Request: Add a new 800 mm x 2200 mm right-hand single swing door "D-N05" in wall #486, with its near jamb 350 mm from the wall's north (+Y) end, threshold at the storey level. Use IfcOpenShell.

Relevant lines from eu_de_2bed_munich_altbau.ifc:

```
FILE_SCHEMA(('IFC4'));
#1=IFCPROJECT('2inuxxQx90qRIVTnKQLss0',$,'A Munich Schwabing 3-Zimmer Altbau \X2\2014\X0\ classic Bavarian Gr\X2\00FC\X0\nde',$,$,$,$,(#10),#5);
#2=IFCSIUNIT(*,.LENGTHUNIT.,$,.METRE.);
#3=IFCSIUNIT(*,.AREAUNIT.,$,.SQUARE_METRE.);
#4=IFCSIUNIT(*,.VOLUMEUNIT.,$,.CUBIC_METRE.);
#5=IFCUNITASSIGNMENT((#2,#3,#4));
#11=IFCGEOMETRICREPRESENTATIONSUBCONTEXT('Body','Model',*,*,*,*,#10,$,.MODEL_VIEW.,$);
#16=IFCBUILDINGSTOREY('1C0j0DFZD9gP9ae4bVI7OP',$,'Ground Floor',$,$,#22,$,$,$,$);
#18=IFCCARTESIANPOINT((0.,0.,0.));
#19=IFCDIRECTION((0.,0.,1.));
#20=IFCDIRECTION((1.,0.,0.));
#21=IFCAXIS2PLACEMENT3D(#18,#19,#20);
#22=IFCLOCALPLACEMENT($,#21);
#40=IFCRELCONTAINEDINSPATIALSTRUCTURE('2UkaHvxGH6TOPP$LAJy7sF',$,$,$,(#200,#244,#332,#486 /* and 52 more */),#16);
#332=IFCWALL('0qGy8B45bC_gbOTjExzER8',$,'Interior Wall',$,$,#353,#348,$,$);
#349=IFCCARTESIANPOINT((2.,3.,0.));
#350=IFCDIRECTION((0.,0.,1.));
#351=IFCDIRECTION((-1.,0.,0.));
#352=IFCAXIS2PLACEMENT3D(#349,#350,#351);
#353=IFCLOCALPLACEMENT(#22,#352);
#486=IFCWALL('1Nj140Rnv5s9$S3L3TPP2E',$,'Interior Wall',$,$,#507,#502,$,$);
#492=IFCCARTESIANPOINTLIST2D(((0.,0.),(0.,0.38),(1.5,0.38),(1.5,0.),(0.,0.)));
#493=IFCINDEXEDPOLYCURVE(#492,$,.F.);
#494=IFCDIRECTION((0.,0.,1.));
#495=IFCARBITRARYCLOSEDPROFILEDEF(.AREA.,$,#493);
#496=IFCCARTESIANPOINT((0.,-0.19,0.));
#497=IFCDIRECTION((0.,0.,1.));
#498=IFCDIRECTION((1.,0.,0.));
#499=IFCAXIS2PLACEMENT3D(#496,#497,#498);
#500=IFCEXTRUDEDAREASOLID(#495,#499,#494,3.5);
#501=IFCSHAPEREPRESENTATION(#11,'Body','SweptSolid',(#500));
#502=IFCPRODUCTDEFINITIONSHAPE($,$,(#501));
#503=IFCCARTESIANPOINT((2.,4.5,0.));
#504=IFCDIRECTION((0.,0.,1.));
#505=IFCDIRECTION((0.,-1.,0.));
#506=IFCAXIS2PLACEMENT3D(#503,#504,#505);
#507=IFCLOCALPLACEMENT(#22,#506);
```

```python
import numpy as np
import ifcopenshell
import ifcopenshell.api.feature
import ifcopenshell.api.geometry
import ifcopenshell.api.root
import ifcopenshell.api.spatial
import ifcopenshell.geom
import ifcopenshell.util.element
import ifcopenshell.util.placement
import ifcopenshell.util.representation
import ifcopenshell.util.shape
import ifcopenshell.util.unit

model = ifcopenshell.open("eu_de_2bed_munich_altbau.ifc")
unit_scale = ifcopenshell.util.unit.calculate_unit_scale(model)
settings = ifcopenshell.geom.settings()


def volume(element):
    """Net volume in cubic metres, openings subtracted."""
    shape = ifcopenshell.geom.create_shape(settings, element)
    return ifcopenshell.util.shape.get_volume(shape.geometry)


wall = model.by_id(486)
storey = ifcopenshell.util.element.get_container(wall, ifc_class="IfcBuildingStorey")
context = ifcopenshell.util.representation.get_context(model, "Model", "Body", "MODEL_VIEW")
before = volume(wall)

width, height, from_end, sill = 0.8, 2.2, 0.35, 0.0  # metres

# The wall runs along its own X axis, and the end named is its -X end.
wall_shape = ifcopenshell.geom.create_shape(settings, wall)
x, y, z = ifcopenshell.util.shape.get_vertices(wall_shape.geometry).T
start = x.min() + from_end
face, thickness = float(y.min()), float(y.max() - y.min())
wall_matrix = ifcopenshell.util.placement.get_local_placement(wall.ObjectPlacement)
level = ifcopenshell.util.placement.get_local_placement(storey.ObjectPlacement)[2, 3]


def in_wall(x, y):
    """Placement at x, y metres in the wall's axes, at sill height."""
    matrix = wall_matrix.copy()
    matrix[:, 3] = wall_matrix @ np.array([x / unit_scale, y / unit_scale, 0.0, 1.0])
    matrix[2, 3] = level + sill / unit_scale
    return matrix


# Opening: a box that overshoots both wall faces by 50 mm.
opening = ifcopenshell.api.root.create_entity(model, ifc_class="IfcOpeningElement", predefined_type="OPENING")
box = ifcopenshell.api.geometry.add_wall_representation(
    model, context=context, length=width, height=height, thickness=thickness + 0.1
)
ifcopenshell.api.geometry.assign_representation(model, product=opening, representation=box)
ifcopenshell.api.geometry.edit_object_placement(model, product=opening, matrix=in_wall(start, face - 0.05), is_si=False)
ifcopenshell.api.feature.add_feature(model, feature=opening, element=wall)

door = ifcopenshell.api.root.create_entity(model, ifc_class="IfcDoor", name="D-N05", predefined_type="DOOR")
door.OverallWidth, door.OverallHeight = width / unit_scale, height / unit_scale
door.OperationType = "SINGLE_SWING_RIGHT"
body = ifcopenshell.api.geometry.add_door_representation(
    model,
    context=context,
    overall_width=door.OverallWidth,
    overall_height=door.OverallHeight,
    operation_type="SINGLE_SWING_RIGHT",
    lining_properties={"LiningDepth": thickness / unit_scale, "ThresholdDepth": thickness / unit_scale},
)
ifcopenshell.api.geometry.assign_representation(model, product=door, representation=body)
ifcopenshell.api.spatial.assign_container(model, products=[door], relating_structure=storey)
ifcopenshell.api.feature.add_filling(model, opening=opening, element=door)

# The lining spans the wall, so the door starts at the wall face.
ifcopenshell.api.geometry.edit_object_placement(model, product=door, matrix=in_wall(start, face), is_si=False)

after = volume(wall)

print(f"wall volume {before:.3f} -> {after:.3f} m3")

model.write("eu_de_2bed_munich_altbau_rev.ifc")
```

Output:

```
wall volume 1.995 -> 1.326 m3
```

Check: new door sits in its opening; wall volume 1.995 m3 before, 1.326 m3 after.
